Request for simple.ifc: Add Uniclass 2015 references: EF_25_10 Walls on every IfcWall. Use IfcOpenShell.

First a look at what the model holds.

```python
import ifcopenshell

model = ifcopenshell.open("simple.ifc")
print(model.schema)
print("classifications:", [c.Name for c in model.by_type("IfcClassification")])
for ifc_class in ("IfcDoor", "IfcRoof", "IfcStair", "IfcWall", "IfcWindow"):
    print(ifc_class, len(model.by_type(ifc_class)))
```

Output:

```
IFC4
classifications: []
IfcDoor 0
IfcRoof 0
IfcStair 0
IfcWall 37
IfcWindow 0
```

```python
import ifcopenshell
import ifcopenshell.api.classification

model = ifcopenshell.open("simple.ifc")

system = ifcopenshell.api.classification.add_classification(model, classification="Uniclass 2015")

codes = {
    "IfcWall": ("EF_25_10", "Walls"),
}
for ifc_class, (code, name) in codes.items():
    products = model.by_type(ifc_class)
    ifcopenshell.api.classification.add_reference(
        model, products=products, classification=system, identification=code, name=name
    )
    print(code, len(products))

model.write("simple_updated.ifc")
```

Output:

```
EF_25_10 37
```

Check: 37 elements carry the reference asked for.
